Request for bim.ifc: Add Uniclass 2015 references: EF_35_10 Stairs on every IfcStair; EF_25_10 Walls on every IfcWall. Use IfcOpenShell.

First a look at what the model holds.

```python
import ifcopenshell

model = ifcopenshell.open("bim.ifc")
print(model.schema)
print("classifications:", [c.Name for c in model.by_type("IfcClassification")])
for ifc_class in ("IfcDoor", "IfcRoof", "IfcStair", "IfcWall", "IfcWindow"):
    print(ifc_class, len(model.by_type(ifc_class)))
```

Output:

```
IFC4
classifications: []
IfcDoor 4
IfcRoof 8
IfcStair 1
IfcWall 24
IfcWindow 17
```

```python
import ifcopenshell
import ifcopenshell.api.classification

model = ifcopenshell.open("bim.ifc")

system = ifcopenshell.api.classification.add_classification(model, classification="Uniclass 2015")

codes = {
    "IfcStair": ("EF_35_10", "Stairs"),
    "IfcWall": ("EF_25_10", "Walls"),
}
for ifc_class, (code, name) in codes.items():
    products = model.by_type(ifc_class)
    ifcopenshell.api.classification.add_reference(
        model, products=products, classification=system, identification=code, name=name
    )
    print(code, len(products))

model.write("bim_updated.ifc")
```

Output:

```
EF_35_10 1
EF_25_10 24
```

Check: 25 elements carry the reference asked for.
